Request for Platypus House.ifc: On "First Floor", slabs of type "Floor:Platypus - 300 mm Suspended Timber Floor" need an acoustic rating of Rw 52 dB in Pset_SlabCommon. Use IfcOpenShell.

First a look at what the model holds.

```python
import ifcopenshell
import ifcopenshell.util.element

model = ifcopenshell.open("Platypus House.ifc")
print(model.schema)
storey = next(s for s in model.by_type("IfcBuildingStorey") if s.Name == "First Floor")
slabs = [e for e in ifcopenshell.util.element.get_decomposition(storey) if e.is_a("IfcSlab")]
seen = {}
for e in slabs:
    element_type = ifcopenshell.util.element.get_type(e)
    key = (element_type.Name if element_type != e and element_type else None, ifcopenshell.util.element.get_pset(e, "Pset_SlabCommon", "AcousticRating"))
    seen[key] = seen.get(key, 0) + 1
for (name, value), count in sorted(seen.items(), key=str):
    print(count, "x", name, "|", value)
```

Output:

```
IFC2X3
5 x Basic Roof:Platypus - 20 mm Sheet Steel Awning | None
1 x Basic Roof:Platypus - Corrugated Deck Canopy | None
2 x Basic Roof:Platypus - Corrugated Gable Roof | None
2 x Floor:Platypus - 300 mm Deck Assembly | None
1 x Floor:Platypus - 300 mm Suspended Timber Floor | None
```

```python
import ifcopenshell
import ifcopenshell.api.pset
import ifcopenshell.util.element

model = ifcopenshell.open("Platypus House.ifc")

storey = next(s for s in model.by_type("IfcBuildingStorey") if s.Name == "First Floor")
slabs = [e for e in ifcopenshell.util.element.get_decomposition(storey) if e.is_a("IfcSlab")]

count = 0
for e in slabs:
    element_type = ifcopenshell.util.element.get_type(e)
    if element_type in (None, e) or element_type.Name != "Floor:Platypus - 300 mm Suspended Timber Floor":
        continue
    # add_pset returns the element's existing set when there is one.
    pset = ifcopenshell.api.pset.add_pset(model, product=e, name="Pset_SlabCommon")
    ifcopenshell.api.pset.edit_pset(model, pset=pset, properties={"AcousticRating": "Rw 52 dB"})
    count += 1

print(count, "slabs updated")

model.write("Platypus House_updated.ifc")
```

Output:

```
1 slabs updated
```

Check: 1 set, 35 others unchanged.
